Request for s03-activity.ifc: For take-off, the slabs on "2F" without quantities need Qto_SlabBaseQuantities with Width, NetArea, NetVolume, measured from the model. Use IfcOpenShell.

First a look at what the model holds.

```python
import ifcopenshell
import ifcopenshell.util.element
import ifcopenshell.util.unit

model = ifcopenshell.open("s03-activity.ifc")
print(model.schema)
for unit_type in ("LENGTHUNIT", "AREAUNIT", "VOLUMEUNIT"):
    print(unit_type, ifcopenshell.util.unit.calculate_unit_scale(model, unit_type))
storey = next(s for s in model.by_type("IfcBuildingStorey") if s.Name == "2F")
slabs = [e for e in ifcopenshell.util.element.get_decomposition(storey) if e.is_a("IfcSlab")]
for e in sorted(slabs, key=lambda e: e.id()):
    print(e.id(), e.is_a(), e.Name, list(ifcopenshell.util.element.get_psets(e, qtos_only=True)), sep=" | ")
```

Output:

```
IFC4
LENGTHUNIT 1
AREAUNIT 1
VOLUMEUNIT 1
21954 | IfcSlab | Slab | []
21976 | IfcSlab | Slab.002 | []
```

```python
import ifcopenshell
import ifcopenshell.api.pset
import ifcopenshell.geom
import ifcopenshell.util.element
import ifcopenshell.util.shape
import ifcopenshell.util.unit

model = ifcopenshell.open("s03-activity.ifc")
unit_scale = ifcopenshell.util.unit.calculate_unit_scale(model)
area_scale = ifcopenshell.util.unit.calculate_unit_scale(model, "AREAUNIT")
volume_scale = ifcopenshell.util.unit.calculate_unit_scale(model, "VOLUMEUNIT")
settings = ifcopenshell.geom.settings()

storey = next(s for s in model.by_type("IfcBuildingStorey") if s.Name == "2F")
slabs = [e for e in ifcopenshell.util.element.get_decomposition(storey) if e.is_a("IfcSlab")]

for e in sorted(slabs, key=lambda e: e.id()):
    if ifcopenshell.util.element.get_psets(e, qtos_only=True, should_inherit=False):
        continue
    # Geometry comes back in metres, in the element's own axes.
    shape = ifcopenshell.geom.create_shape(settings, e)
    values = {
        "Width": ifcopenshell.util.shape.get_z(shape.geometry) / unit_scale,
        "NetArea": ifcopenshell.util.shape.get_footprint_area(shape.geometry) / area_scale,
        "NetVolume": ifcopenshell.util.shape.get_volume(shape.geometry) / volume_scale,
    }
    qto = ifcopenshell.api.pset.add_qto(model, product=e, name="Qto_SlabBaseQuantities")
    ifcopenshell.api.pset.edit_qto(model, qto=qto, properties=values)
    print(e.id(), {k: round(v, 3) for k, v in values.items()})

model.write("s03-activity-out.ifc")
```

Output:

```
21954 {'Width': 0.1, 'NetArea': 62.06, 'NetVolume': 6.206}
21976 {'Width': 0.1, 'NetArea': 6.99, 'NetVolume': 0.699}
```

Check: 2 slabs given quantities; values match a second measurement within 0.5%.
